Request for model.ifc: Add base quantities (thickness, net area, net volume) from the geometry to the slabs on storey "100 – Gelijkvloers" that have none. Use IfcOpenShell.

First a look at what the model holds.

```python
import ifcopenshell
import ifcopenshell.util.element
import ifcopenshell.util.unit

model = ifcopenshell.open("model.ifc")
print(model.schema)
for unit_type in ("LENGTHUNIT", "AREAUNIT", "VOLUMEUNIT"):
    print(unit_type, ifcopenshell.util.unit.calculate_unit_scale(model, unit_type))
storey = next(s for s in model.by_type("IfcBuildingStorey") if s.Name == "100 – Gelijkvloers")
slabs = [e for e in ifcopenshell.util.element.get_decomposition(storey) if e.is_a("IfcSlab")]
for e in sorted(slabs, key=lambda e: e.id()):
    print(e.id(), e.is_a(), e.Name, list(ifcopenshell.util.element.get_psets(e, qtos_only=True)), sep=" | ")
```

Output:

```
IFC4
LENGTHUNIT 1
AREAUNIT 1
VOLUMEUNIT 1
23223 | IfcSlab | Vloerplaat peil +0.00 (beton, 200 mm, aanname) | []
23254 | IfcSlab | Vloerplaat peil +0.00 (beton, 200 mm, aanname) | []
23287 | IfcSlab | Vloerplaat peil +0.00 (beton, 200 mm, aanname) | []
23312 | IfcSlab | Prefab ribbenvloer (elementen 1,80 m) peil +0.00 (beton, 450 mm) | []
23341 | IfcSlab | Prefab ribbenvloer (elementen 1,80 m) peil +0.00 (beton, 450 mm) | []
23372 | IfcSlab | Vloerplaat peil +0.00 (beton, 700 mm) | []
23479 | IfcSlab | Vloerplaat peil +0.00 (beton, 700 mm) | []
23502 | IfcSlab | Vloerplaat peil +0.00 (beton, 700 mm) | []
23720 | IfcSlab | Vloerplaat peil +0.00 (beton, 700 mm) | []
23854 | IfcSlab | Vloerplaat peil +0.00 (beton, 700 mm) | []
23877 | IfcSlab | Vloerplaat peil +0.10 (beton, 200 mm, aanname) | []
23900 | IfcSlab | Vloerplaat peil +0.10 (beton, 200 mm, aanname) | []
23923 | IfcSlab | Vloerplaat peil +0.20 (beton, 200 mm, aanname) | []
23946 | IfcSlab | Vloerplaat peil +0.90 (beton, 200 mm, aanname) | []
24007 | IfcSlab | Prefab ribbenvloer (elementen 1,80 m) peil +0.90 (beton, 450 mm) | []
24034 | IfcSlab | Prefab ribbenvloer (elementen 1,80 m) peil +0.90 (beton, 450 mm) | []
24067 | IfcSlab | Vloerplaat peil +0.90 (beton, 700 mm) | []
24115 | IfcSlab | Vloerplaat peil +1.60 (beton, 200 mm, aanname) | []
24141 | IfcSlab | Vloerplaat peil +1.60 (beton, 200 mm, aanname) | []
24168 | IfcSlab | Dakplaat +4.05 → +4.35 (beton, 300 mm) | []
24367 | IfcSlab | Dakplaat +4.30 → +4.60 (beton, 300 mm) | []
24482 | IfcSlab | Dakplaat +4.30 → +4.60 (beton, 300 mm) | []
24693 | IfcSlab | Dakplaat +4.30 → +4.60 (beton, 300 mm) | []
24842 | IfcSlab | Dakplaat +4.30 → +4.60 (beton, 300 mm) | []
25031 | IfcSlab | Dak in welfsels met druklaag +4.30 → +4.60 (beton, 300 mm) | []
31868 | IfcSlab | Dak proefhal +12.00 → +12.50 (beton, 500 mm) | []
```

```python
import ifcopenshell
import ifcopenshell.api.pset
import ifcopenshell.geom
import ifcopenshell.util.element
import ifcopenshell.util.shape
import ifcopenshell.util.unit

model = ifcopenshell.open("model.ifc")
unit_scale = ifcopenshell.util.unit.calculate_unit_scale(model)
area_scale = ifcopenshell.util.unit.calculate_unit_scale(model, "AREAUNIT")
volume_scale = ifcopenshell.util.unit.calculate_unit_scale(model, "VOLUMEUNIT")
settings = ifcopenshell.geom.settings()

storey = next(s for s in model.by_type("IfcBuildingStorey") if s.Name == "100 – Gelijkvloers")
slabs = [e for e in ifcopenshell.util.element.get_decomposition(storey) if e.is_a("IfcSlab")]

for e in sorted(slabs, key=lambda e: e.id()):
    if ifcopenshell.util.element.get_psets(e, qtos_only=True, should_inherit=False):
        continue
    # Geometry comes back in metres, in the element's own axes.
    shape = ifcopenshell.geom.create_shape(settings, e)
    values = {
        "Width": ifcopenshell.util.shape.get_z(shape.geometry) / unit_scale,
        "NetArea": ifcopenshell.util.shape.get_footprint_area(shape.geometry) / area_scale,
        "NetVolume": ifcopenshell.util.shape.get_volume(shape.geometry) / volume_scale,
    }
    qto = ifcopenshell.api.pset.add_qto(model, product=e, name="Qto_SlabBaseQuantities")
    ifcopenshell.api.pset.edit_qto(model, qto=qto, properties=values)
    print(e.id(), {k: round(v, 3) for k, v in values.items()})

model.write("model_rev.ifc")
```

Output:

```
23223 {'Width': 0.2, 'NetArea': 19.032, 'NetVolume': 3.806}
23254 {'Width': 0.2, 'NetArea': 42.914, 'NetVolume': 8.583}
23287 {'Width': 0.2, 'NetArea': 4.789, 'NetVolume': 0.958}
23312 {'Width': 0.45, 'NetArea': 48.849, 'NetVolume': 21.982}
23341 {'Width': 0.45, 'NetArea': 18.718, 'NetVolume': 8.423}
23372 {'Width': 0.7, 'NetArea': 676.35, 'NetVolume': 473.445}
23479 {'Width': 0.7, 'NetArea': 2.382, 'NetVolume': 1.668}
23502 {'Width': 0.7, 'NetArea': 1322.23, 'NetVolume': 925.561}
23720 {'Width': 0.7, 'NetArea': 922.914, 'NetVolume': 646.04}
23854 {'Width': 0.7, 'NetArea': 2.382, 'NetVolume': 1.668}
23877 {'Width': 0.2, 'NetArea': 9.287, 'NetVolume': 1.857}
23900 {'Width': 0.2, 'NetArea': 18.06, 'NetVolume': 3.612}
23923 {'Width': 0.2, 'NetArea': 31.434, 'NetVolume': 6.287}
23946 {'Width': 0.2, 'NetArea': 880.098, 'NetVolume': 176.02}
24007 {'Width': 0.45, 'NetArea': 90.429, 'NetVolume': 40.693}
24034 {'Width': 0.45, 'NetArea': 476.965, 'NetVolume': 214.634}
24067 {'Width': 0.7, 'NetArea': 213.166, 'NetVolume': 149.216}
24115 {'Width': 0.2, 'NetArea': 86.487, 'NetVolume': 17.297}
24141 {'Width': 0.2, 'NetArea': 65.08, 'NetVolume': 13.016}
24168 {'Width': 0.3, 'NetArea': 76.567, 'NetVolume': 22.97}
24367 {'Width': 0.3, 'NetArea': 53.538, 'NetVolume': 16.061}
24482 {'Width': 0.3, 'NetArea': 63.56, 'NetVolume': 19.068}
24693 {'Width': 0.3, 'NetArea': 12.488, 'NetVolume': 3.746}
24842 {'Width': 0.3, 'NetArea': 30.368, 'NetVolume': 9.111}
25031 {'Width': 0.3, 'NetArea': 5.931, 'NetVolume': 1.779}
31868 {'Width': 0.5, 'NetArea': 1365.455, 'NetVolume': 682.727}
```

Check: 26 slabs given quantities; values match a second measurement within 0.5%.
